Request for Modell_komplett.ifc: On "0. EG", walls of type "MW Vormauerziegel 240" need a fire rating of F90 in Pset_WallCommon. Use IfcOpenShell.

First a look at what the model holds.

```python
import ifcopenshell
import ifcopenshell.util.element

model = ifcopenshell.open("Modell_komplett.ifc")
print(model.schema)
storey = next(s for s in model.by_type("IfcBuildingStorey") if s.Name == "0. EG")
walls = [e for e in ifcopenshell.util.element.get_decomposition(storey) if e.is_a("IfcWall")]
seen = {}
for e in walls:
    element_type = ifcopenshell.util.element.get_type(e)
    key = (element_type.Name if element_type != e and element_type else None, ifcopenshell.util.element.get_pset(e, "Pset_WallCommon", "FireRating"))
    seen[key] = seen.get(key, 0) + 1
for (name, value), count in sorted(seen.items(), key=str):
    print(count, "x", name, "|", value)
```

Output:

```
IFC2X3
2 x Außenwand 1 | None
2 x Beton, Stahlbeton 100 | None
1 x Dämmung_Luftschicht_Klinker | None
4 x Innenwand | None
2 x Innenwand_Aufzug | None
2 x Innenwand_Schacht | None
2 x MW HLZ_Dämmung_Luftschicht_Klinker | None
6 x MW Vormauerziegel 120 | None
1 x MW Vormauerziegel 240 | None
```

```python
import ifcopenshell
import ifcopenshell.api.pset
import ifcopenshell.util.element

model = ifcopenshell.open("Modell_komplett.ifc")

storey = next(s for s in model.by_type("IfcBuildingStorey") if s.Name == "0. EG")
walls = [e for e in ifcopenshell.util.element.get_decomposition(storey) if e.is_a("IfcWall")]

count = 0
for e in walls:
    element_type = ifcopenshell.util.element.get_type(e)
    if element_type in (None, e) or element_type.Name != "MW Vormauerziegel 240":
        continue
    # add_pset returns the element's existing set when there is one.
    pset = ifcopenshell.api.pset.add_pset(model, product=e, name="Pset_WallCommon")
    ifcopenshell.api.pset.edit_pset(model, pset=pset, properties={"FireRating": "F90"})
    count += 1

print(count, "walls updated")

model.write("Modell_komplett-out.ifc")
```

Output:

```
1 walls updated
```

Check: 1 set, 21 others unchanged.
